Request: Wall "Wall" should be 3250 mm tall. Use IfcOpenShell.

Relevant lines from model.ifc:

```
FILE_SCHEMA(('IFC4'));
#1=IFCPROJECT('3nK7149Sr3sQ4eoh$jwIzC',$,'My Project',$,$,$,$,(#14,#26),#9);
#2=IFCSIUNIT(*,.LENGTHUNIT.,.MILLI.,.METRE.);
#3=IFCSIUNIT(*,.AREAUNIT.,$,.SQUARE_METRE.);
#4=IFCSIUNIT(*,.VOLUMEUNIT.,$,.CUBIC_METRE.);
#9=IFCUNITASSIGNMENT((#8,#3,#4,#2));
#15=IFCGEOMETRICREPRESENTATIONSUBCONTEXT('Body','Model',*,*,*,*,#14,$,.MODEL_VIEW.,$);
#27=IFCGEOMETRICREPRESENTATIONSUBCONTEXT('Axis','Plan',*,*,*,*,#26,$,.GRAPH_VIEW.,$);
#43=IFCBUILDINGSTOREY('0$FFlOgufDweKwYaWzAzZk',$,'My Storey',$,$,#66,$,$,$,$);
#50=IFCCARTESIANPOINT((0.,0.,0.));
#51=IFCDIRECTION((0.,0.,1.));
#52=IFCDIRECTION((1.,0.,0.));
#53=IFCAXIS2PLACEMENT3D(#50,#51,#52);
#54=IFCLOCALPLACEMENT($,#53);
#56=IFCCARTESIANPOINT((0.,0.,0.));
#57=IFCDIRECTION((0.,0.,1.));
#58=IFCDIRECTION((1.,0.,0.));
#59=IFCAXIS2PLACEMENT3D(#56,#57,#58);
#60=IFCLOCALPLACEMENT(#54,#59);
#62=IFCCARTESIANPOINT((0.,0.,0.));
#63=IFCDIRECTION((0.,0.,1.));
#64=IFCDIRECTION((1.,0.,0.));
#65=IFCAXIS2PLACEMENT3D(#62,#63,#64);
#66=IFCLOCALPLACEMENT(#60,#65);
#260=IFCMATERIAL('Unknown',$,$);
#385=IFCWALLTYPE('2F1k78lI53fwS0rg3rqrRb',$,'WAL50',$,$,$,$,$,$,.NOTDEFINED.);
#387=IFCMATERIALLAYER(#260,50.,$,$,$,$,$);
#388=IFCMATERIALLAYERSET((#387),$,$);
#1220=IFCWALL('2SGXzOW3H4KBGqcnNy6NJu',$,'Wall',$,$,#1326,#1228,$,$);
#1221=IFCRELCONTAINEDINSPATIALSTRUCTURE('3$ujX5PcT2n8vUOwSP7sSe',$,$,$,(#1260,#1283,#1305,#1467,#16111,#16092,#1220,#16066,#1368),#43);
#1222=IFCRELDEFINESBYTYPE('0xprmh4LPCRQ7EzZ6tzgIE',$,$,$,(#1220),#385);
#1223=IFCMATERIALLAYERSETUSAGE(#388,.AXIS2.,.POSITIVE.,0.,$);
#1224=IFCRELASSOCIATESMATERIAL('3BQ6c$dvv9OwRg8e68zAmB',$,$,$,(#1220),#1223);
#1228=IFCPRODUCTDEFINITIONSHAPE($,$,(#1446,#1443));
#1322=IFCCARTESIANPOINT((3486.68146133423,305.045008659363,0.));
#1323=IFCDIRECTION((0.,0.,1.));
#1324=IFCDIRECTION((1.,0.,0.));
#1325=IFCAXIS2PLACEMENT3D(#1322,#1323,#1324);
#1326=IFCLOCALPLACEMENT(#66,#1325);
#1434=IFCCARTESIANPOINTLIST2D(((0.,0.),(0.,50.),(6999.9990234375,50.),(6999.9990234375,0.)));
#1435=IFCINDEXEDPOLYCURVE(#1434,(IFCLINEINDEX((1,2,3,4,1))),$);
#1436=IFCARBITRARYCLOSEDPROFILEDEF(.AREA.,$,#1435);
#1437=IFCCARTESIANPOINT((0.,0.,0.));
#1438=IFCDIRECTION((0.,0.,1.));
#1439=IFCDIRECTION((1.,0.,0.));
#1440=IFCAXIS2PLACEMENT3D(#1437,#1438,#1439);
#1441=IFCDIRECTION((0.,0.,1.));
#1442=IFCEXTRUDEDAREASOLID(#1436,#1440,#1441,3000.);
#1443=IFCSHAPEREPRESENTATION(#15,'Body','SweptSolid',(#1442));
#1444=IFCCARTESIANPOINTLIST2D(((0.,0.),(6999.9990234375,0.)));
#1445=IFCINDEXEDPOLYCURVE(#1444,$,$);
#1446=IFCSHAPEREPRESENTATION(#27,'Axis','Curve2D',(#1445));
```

```python
import ifcopenshell
import ifcopenshell.geom
import ifcopenshell.util.representation
import ifcopenshell.util.shape
import ifcopenshell.util.unit

model = ifcopenshell.open("model.ifc")
unit_scale = ifcopenshell.util.unit.calculate_unit_scale(model)
settings = ifcopenshell.geom.settings()


def volume(element):
    """Net volume in cubic metres, openings subtracted."""
    shape = ifcopenshell.geom.create_shape(settings, element)
    return ifcopenshell.util.shape.get_volume(shape.geometry)


wall = model.by_guid("2SGXzOW3H4KBGqcnNy6NJu")
before = volume(wall)

body = ifcopenshell.util.representation.get_representation(wall, "Model", "Body")
solid = body.Items[0]
old_height = solid.Depth
solid.Depth = 3.25 / unit_scale
after = volume(wall)

print(f"height {old_height:g} -> {solid.Depth:g}, volume {before:.3f} -> {after:.3f} m3")

model.write("model-out.ifc")
```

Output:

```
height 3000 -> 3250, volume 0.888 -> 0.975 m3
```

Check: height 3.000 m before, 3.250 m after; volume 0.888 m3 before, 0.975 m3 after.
